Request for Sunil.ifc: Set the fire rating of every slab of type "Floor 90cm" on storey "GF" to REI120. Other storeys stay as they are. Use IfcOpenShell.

First a look at what the model holds.

```python
import ifcopenshell
import ifcopenshell.util.element

model = ifcopenshell.open("Sunil.ifc")
print(model.schema)
storey = next(s for s in model.by_type("IfcBuildingStorey") if s.Name == "GF")
slabs = [e for e in ifcopenshell.util.element.get_decomposition(storey) if e.is_a("IfcSlab")]
seen = {}
for e in slabs:
    element_type = ifcopenshell.util.element.get_type(e)
    key = (element_type.Name if element_type != e and element_type else None, ifcopenshell.util.element.get_pset(e, "Pset_SlabCommon", "FireRating"))
    seen[key] = seen.get(key, 0) + 1
for (name, value), count in sorted(seen.items(), key=str):
    print(count, "x", name, "|", value)
```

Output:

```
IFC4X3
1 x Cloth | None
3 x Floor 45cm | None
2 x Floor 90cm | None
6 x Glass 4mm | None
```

```python
import ifcopenshell
import ifcopenshell.api.pset
import ifcopenshell.util.element

model = ifcopenshell.open("Sunil.ifc")

storey = next(s for s in model.by_type("IfcBuildingStorey") if s.Name == "GF")
slabs = [e for e in ifcopenshell.util.element.get_decomposition(storey) if e.is_a("IfcSlab")]

count = 0
for e in slabs:
    element_type = ifcopenshell.util.element.get_type(e)
    if element_type in (None, e) or element_type.Name != "Floor 90cm":
        continue
    # add_pset returns the element's existing set when there is one.
    pset = ifcopenshell.api.pset.add_pset(model, product=e, name="Pset_SlabCommon")
    ifcopenshell.api.pset.edit_pset(model, pset=pset, properties={"FireRating": "REI120"})
    count += 1

print(count, "slabs updated")

model.write("Sunil_edited.ifc")
```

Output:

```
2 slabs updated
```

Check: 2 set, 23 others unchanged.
